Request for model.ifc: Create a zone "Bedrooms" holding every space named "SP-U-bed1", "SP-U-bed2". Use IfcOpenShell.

First a look at what the model holds.

```python
import ifcopenshell

model = ifcopenshell.open("model.ifc")
print(model.schema)
seen = {}
for space in model.by_type("IfcSpace"):
    seen[space.LongName] = seen.get(space.LongName, 0) + 1
for name, count in sorted(seen.items(), key=str):
    print(count, "x", name)
print("zones:", [z.Name for z in model.by_type("IfcZone")][:20])
```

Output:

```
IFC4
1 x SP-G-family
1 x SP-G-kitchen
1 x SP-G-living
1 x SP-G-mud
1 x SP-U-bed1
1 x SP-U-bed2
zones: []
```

```python
import ifcopenshell
import ifcopenshell.api.group
import ifcopenshell.api.root

model = ifcopenshell.open("model.ifc")

names = {"SP-U-bed1", "SP-U-bed2"}
spaces = [s for s in model.by_type("IfcSpace") if s.LongName in names]

zone = ifcopenshell.api.root.create_entity(model, ifc_class="IfcZone", name="Bedrooms")
ifcopenshell.api.group.assign_group(model, products=spaces, group=zone)
print(len(spaces), "spaces in", zone.Name)

model.write("model-out.ifc")
```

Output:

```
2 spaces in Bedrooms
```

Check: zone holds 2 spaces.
